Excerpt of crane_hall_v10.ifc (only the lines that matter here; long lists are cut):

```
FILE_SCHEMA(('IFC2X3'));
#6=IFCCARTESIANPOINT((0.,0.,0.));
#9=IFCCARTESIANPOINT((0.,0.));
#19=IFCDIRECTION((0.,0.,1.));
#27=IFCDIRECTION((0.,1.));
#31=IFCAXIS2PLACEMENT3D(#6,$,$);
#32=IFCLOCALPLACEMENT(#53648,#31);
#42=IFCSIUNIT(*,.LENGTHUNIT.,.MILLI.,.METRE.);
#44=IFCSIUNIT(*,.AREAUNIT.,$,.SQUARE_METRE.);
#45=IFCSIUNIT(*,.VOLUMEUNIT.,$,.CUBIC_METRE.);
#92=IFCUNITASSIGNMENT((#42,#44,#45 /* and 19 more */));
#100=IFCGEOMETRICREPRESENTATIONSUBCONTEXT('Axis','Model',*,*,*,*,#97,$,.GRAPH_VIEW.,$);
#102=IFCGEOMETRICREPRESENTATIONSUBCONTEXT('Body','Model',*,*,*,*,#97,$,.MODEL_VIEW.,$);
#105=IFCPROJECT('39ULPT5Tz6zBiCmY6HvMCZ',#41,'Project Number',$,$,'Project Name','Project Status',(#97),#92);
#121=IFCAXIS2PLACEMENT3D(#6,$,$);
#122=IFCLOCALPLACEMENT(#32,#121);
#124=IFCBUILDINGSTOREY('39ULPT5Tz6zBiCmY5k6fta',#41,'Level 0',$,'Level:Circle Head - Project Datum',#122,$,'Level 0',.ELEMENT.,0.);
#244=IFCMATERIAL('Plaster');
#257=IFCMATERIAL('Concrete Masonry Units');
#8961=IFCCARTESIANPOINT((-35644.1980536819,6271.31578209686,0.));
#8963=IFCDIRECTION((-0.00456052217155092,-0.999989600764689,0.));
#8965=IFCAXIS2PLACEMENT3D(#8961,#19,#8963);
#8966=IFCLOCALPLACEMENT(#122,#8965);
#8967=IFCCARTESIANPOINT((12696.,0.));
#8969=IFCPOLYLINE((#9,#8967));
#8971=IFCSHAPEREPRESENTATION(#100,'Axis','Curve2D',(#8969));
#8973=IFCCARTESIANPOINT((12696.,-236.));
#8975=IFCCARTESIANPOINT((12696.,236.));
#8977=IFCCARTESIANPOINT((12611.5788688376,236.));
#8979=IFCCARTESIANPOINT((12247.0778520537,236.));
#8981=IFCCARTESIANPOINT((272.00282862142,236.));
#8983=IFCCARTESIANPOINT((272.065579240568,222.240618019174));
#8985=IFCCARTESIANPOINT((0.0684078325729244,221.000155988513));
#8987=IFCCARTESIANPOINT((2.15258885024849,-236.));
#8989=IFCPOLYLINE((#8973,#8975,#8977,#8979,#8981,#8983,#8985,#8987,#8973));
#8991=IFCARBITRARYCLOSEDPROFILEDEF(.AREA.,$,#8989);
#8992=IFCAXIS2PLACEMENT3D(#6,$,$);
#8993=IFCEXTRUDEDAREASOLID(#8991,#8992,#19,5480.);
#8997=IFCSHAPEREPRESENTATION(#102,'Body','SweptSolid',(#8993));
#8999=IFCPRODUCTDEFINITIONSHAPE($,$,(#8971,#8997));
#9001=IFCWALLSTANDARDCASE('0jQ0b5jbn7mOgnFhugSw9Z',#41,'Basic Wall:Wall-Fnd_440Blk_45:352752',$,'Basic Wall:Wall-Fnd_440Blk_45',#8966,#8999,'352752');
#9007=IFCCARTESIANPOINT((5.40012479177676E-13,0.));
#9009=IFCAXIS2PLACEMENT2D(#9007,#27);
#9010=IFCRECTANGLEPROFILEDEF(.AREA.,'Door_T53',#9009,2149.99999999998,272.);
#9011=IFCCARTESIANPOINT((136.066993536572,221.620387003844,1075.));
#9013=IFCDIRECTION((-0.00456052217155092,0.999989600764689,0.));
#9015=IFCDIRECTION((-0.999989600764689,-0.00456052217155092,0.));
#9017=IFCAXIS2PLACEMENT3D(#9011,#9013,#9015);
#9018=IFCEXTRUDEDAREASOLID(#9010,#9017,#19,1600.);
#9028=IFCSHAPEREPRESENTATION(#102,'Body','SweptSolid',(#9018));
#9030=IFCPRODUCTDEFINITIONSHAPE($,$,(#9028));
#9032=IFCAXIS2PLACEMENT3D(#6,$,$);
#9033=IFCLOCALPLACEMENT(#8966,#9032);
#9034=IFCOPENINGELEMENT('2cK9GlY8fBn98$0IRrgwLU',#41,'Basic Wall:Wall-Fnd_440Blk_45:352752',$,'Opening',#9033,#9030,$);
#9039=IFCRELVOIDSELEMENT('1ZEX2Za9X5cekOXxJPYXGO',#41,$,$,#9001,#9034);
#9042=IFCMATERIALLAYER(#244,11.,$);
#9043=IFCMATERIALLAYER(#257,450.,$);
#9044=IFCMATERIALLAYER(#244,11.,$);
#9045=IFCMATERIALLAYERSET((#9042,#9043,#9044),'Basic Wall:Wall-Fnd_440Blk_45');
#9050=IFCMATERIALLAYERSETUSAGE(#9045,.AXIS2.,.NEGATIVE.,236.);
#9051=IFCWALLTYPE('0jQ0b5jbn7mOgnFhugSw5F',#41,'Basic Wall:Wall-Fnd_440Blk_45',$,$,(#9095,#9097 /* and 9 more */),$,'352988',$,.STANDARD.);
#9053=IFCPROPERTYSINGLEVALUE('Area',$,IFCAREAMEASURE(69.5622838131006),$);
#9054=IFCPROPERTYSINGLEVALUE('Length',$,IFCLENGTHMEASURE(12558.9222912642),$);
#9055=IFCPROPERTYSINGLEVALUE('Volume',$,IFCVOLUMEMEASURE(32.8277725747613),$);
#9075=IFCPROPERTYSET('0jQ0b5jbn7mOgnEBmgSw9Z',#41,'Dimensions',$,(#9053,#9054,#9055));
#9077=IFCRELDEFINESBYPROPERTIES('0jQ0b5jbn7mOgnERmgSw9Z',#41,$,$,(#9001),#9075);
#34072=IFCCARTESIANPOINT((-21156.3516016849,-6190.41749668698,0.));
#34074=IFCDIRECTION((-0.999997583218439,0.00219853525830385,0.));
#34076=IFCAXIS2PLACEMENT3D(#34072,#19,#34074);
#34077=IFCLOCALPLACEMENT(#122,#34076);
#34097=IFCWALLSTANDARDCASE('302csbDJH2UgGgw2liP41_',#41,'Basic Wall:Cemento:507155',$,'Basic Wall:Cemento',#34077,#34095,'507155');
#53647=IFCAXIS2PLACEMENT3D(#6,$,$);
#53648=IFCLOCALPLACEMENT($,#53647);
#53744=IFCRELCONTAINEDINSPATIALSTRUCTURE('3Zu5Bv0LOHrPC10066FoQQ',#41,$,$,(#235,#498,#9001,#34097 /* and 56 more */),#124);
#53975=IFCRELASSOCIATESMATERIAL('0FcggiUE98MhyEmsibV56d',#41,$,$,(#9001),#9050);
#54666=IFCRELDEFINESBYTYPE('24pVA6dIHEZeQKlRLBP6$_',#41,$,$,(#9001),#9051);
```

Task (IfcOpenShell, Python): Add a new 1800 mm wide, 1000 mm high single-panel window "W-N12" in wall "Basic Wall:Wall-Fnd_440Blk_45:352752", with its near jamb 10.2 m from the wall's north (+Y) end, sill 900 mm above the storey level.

```python
import numpy as np
import ifcopenshell
import ifcopenshell.api.feature
import ifcopenshell.api.geometry
import ifcopenshell.api.pset
import ifcopenshell.api.root
import ifcopenshell.api.spatial
import ifcopenshell.api.type
import ifcopenshell.geom
import ifcopenshell.util.element
import ifcopenshell.util.placement
import ifcopenshell.util.representation
import ifcopenshell.util.shape
import ifcopenshell.util.unit

model = ifcopenshell.open("crane_hall_v10.ifc")
unit_scale = ifcopenshell.util.unit.calculate_unit_scale(model)
area_scale = ifcopenshell.util.unit.calculate_unit_scale(model, "AREAUNIT")
volume_scale = ifcopenshell.util.unit.calculate_unit_scale(model, "VOLUMEUNIT")
settings = ifcopenshell.geom.settings()


def volume(element):
    """Net volume in cubic metres, openings subtracted."""
    shape = ifcopenshell.geom.create_shape(settings, element)
    return ifcopenshell.util.shape.get_volume(shape.geometry)


wall = model.by_guid("0jQ0b5jbn7mOgnFhugSw9Z")
storey = ifcopenshell.util.element.get_container(wall, ifc_class="IfcBuildingStorey")
context = ifcopenshell.util.representation.get_context(model, "Model", "Body", "MODEL_VIEW")
before = volume(wall)

width, height, from_end, sill = 1.8, 1, 10.2, 0.9  # metres

# The wall runs along its own X axis, and the end named is its -X end.
wall_shape = ifcopenshell.geom.create_shape(settings, wall)
x, y, z = ifcopenshell.util.shape.get_vertices(wall_shape.geometry).T
start = x.min() + from_end
face, thickness = float(y.min()), float(y.max() - y.min())
wall_matrix = ifcopenshell.util.placement.get_local_placement(wall.ObjectPlacement)
level = ifcopenshell.util.placement.get_local_placement(storey.ObjectPlacement)[2, 3]


def in_wall(x, y):
    """Placement at x, y metres in the wall's axes, at sill height."""
    matrix = wall_matrix.copy()
    matrix[:, 3] = wall_matrix @ np.array([x / unit_scale, y / unit_scale, 0.0, 1.0])
    matrix[2, 3] = level + sill / unit_scale
    return matrix


# Opening: a box that overshoots both wall faces by 50 mm.
opening = ifcopenshell.api.root.create_entity(model, ifc_class="IfcOpeningElement")
box = ifcopenshell.api.geometry.add_wall_representation(
    model, context=context, length=width, height=height, thickness=thickness + 0.1
)
ifcopenshell.api.geometry.assign_representation(model, product=opening, representation=box)
ifcopenshell.api.geometry.edit_object_placement(model, product=opening, matrix=in_wall(start, face - 0.05), is_si=False)
ifcopenshell.api.feature.add_feature(model, feature=opening, element=wall)

window = ifcopenshell.api.root.create_entity(model, ifc_class="IfcWindow", name="W-N12")
window.OverallWidth, window.OverallHeight = width / unit_scale, height / unit_scale
body = ifcopenshell.api.geometry.add_window_representation(
    model,
    context=context,
    overall_width=window.OverallWidth,
    overall_height=window.OverallHeight,
    partition_type="SINGLE_PANEL",
)
ifcopenshell.api.geometry.assign_representation(model, product=window, representation=body)
ifcopenshell.api.spatial.assign_container(model, products=[window], relating_structure=storey)
fills = ifcopenshell.api.feature.add_filling(model, opening=opening, element=window)
fills.OwnerHistory = window.OwnerHistory  # required in IFC2X3

# IFC2X3 keeps the operation on the window style.
style = ifcopenshell.api.root.create_entity(model, ifc_class="IfcWindowStyle", name="W-N12")
style.OperationType, style.ConstructionType = "SINGLE_PANEL", "NOTDEFINED"
style.ParameterTakesPrecedence = style.Sizeable = False
ifcopenshell.api.type.assign_type(model, related_objects=[window], relating_type=style)

# Centre the window in the wall's thickness.
ifcopenshell.api.geometry.edit_object_placement(model, product=window, matrix=in_wall(start, face), is_si=False)
window_shape = ifcopenshell.geom.create_shape(settings, window)
depth = ifcopenshell.util.shape.get_vertices(window_shape.geometry)[:, 1]
offset = face + thickness / 2 - (depth.min() + depth.max()) / 2
ifcopenshell.api.geometry.edit_object_placement(model, product=window, matrix=in_wall(start, offset), is_si=False)

after = volume(wall)

# Update the wall's stored quantities.
pset = model.by_id(ifcopenshell.util.element.get_pset(wall, "Dimensions", should_inherit=False)["id"])
ifcopenshell.api.pset.edit_pset(model, pset=pset, properties={
    "Area": model.create_entity("IfcAreaMeasure", after / thickness / area_scale),
    "Volume": model.create_entity("IfcVolumeMeasure", after / volume_scale),
})

print(f"wall volume {before:.3f} -> {after:.3f} m3")

model.write("crane_hall_v10-out.ifc")
```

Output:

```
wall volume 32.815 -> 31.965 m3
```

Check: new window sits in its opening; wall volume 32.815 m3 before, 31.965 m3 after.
